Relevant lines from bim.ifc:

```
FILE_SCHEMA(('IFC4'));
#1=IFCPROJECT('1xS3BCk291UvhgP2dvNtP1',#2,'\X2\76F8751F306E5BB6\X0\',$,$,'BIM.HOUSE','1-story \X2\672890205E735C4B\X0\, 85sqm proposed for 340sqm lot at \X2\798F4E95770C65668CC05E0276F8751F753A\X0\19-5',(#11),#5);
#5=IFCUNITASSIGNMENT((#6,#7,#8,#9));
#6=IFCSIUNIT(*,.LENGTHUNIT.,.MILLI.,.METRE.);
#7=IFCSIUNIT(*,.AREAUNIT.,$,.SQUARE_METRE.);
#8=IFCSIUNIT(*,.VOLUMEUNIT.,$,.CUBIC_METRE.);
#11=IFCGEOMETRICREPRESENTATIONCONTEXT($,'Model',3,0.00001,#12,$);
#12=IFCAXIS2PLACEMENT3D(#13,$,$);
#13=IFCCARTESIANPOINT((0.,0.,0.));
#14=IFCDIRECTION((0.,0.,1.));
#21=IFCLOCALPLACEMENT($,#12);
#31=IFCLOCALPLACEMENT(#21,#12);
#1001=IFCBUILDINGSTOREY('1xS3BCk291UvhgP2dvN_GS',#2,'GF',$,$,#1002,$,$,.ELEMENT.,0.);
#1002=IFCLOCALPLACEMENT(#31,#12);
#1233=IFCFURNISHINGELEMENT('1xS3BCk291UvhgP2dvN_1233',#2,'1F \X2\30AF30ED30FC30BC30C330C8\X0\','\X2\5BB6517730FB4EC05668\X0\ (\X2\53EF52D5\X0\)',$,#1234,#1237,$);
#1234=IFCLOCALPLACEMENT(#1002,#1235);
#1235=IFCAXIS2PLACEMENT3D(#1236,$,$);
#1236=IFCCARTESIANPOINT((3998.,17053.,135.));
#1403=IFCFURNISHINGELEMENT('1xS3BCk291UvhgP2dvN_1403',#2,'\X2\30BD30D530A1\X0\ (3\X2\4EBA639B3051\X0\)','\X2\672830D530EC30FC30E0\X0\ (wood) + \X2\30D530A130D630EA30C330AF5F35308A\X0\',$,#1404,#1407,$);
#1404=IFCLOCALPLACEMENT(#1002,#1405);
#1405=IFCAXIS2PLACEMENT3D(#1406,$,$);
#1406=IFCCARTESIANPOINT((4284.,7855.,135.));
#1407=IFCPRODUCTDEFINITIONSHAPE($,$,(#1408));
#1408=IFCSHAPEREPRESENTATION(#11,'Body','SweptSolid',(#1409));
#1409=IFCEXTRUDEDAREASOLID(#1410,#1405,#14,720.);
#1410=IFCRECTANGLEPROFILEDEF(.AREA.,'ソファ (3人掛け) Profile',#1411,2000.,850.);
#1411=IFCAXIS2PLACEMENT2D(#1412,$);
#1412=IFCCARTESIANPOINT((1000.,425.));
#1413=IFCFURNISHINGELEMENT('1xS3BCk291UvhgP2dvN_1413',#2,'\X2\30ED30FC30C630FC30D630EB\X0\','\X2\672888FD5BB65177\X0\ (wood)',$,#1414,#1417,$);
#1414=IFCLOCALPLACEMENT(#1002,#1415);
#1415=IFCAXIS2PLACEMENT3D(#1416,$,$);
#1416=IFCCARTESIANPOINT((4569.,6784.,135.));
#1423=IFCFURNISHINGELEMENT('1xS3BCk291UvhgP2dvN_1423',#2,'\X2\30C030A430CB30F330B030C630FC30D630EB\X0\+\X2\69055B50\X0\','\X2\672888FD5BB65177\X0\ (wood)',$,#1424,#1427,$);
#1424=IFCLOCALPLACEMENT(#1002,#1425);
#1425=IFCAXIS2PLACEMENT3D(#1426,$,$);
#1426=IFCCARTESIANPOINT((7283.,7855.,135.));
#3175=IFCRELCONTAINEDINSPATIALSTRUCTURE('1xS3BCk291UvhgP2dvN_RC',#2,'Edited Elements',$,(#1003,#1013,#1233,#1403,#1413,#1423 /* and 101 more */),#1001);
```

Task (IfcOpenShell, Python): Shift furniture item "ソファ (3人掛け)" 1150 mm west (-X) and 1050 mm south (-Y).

```python
import ifcopenshell
import ifcopenshell.api.geometry
import ifcopenshell.util.placement

model = ifcopenshell.open("bim.ifc")

item = model.by_id(1403)
matrix = ifcopenshell.util.placement.get_local_placement(item.ObjectPlacement)
matrix[0, 3] -= 1150.0
matrix[1, 3] -= 1050.0
ifcopenshell.api.geometry.edit_object_placement(model, product=item, matrix=matrix, is_si=False)

print(ifcopenshell.util.placement.get_local_placement(item.ObjectPlacement).round(3) + 0.0)

model.write("bim_rev.ifc")
```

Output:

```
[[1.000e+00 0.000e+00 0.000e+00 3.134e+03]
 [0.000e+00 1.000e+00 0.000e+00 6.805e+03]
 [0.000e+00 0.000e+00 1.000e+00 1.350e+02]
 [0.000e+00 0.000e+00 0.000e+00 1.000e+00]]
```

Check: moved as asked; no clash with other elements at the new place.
